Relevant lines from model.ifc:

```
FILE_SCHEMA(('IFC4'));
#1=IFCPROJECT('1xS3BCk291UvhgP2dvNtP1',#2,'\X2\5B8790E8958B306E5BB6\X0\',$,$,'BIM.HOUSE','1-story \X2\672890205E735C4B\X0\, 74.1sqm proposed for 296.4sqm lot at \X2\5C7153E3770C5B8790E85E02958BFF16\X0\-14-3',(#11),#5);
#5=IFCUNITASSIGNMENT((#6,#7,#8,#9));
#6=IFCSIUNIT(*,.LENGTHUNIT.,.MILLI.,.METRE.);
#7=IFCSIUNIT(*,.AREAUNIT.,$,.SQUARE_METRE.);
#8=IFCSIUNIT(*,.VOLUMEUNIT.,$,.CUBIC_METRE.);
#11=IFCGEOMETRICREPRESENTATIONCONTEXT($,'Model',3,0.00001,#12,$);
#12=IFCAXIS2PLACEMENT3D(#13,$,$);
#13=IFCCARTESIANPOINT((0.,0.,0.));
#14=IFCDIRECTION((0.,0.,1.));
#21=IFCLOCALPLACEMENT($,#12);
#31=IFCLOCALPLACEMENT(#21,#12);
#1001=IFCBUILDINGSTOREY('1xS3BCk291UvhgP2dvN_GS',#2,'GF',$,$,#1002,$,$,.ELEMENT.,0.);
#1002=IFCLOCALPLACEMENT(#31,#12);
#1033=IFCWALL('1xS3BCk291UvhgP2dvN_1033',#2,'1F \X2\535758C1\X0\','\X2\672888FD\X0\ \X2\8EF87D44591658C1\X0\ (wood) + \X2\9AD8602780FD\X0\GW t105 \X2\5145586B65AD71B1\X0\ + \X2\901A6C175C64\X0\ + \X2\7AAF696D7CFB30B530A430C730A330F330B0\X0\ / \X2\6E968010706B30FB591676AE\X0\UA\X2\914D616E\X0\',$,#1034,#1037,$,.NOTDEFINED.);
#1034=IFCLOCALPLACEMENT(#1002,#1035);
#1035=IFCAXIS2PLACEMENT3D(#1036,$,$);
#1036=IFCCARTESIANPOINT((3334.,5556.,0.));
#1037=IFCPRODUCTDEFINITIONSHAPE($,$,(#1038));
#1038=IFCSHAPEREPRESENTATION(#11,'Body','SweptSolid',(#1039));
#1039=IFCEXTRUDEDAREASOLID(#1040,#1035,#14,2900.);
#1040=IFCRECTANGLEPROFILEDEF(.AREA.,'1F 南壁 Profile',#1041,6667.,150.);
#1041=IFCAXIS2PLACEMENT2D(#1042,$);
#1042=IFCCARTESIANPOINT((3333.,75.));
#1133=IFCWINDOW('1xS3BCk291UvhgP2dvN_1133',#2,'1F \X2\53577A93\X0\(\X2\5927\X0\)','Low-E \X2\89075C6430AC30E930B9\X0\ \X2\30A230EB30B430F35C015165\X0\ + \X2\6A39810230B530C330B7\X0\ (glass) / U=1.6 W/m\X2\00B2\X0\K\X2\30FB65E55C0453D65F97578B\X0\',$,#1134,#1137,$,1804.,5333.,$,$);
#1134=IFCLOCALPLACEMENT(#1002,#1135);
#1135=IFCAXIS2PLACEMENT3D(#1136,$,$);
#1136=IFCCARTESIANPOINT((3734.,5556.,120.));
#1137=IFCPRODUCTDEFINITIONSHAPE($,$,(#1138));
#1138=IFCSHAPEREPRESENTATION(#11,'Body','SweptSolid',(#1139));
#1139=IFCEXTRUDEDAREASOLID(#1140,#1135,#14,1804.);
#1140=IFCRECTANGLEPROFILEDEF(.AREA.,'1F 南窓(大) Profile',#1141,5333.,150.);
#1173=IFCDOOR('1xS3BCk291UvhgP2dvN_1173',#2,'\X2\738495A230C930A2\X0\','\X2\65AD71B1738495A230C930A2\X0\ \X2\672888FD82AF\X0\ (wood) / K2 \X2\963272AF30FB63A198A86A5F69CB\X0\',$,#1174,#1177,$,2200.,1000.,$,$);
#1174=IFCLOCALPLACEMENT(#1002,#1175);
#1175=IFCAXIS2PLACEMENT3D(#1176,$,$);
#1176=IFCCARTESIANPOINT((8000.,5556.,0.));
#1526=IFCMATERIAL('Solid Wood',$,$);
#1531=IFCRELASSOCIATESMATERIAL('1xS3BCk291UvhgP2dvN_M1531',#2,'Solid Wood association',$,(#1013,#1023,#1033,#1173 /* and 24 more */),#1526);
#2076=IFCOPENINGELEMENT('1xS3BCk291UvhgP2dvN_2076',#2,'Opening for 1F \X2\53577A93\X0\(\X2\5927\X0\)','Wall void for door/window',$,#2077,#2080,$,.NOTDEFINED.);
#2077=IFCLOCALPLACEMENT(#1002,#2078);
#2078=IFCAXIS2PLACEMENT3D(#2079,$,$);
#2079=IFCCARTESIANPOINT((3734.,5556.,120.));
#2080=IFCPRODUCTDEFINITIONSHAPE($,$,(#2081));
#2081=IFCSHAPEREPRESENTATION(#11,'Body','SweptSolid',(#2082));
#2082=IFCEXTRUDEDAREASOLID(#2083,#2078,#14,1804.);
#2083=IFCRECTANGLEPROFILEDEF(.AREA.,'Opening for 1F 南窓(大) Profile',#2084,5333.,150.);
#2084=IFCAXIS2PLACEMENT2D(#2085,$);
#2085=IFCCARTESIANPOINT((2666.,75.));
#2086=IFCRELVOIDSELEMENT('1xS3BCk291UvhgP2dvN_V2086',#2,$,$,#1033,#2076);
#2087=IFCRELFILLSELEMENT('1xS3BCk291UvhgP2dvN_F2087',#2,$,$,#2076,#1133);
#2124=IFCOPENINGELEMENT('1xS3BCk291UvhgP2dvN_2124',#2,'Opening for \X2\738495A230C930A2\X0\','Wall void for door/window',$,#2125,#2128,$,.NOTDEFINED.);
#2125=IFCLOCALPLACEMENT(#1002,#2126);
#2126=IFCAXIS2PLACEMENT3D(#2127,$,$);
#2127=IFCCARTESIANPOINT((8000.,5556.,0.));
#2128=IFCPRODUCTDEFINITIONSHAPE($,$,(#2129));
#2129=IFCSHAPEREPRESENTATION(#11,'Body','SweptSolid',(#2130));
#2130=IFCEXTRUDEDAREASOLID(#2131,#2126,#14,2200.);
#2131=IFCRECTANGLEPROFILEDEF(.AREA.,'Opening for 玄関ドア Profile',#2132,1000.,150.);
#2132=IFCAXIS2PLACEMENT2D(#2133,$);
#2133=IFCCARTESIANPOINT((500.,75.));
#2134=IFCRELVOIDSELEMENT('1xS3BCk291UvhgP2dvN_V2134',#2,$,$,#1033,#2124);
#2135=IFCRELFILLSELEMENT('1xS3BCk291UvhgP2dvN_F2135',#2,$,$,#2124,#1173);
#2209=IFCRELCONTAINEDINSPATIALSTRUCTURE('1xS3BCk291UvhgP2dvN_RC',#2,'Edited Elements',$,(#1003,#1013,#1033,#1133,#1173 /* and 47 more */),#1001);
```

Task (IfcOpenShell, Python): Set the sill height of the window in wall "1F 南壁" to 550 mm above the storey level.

```python
import numpy as np
import ifcopenshell
import ifcopenshell.api.geometry
import ifcopenshell.geom
import ifcopenshell.util.element
import ifcopenshell.util.placement
import ifcopenshell.util.shape
import ifcopenshell.util.unit

model = ifcopenshell.open("model.ifc")
unit_scale = ifcopenshell.util.unit.calculate_unit_scale(model)

window = model.by_guid("1xS3BCk291UvhgP2dvN_1133")
opening = window.FillsVoids[0].RelatingOpeningElement
storey = ifcopenshell.util.element.get_container(window, ifc_class="IfcBuildingStorey")
level = ifcopenshell.util.placement.get_local_placement(storey.ObjectPlacement)[2, 3]

# The opening's origin need not be at the sill, so measure its lowest point.
shape = ifcopenshell.geom.create_shape(ifcopenshell.geom.settings(), opening)
bottom = ifcopenshell.util.shape.get_shape_bottom_elevation(shape, shape.geometry) / unit_scale
dz = level + 550.0 - bottom

shift = np.array([0.0, 0.0, dz])
# The window is not placed relative to its opening, so move both.
for product in (opening, window):
    matrix = ifcopenshell.util.placement.get_local_placement(product.ObjectPlacement)
    matrix[:3, 3] += shift
    ifcopenshell.api.geometry.edit_object_placement(model, product=product, matrix=matrix, is_si=False)

print(f"moved by {dz * unit_scale:+.3f} m")

model.write("model-out.ifc")
```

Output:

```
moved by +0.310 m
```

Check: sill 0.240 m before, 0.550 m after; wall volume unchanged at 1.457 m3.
